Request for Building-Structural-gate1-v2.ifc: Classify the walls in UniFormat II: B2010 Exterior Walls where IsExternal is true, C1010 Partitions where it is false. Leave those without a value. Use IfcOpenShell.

First a look at what the model holds.

```python
import ifcopenshell
import ifcopenshell.util.element

model = ifcopenshell.open("Building-Structural-gate1-v2.ifc")
print(model.schema)
print("classifications:", [c.Name for c in model.by_type("IfcClassification")])
values = [ifcopenshell.util.element.get_pset(e, "Pset_WallCommon", "IsExternal") for e in model.by_type("IfcWall")]
for value in (True, False, None):
    print("IsExternal", value, values.count(value))
```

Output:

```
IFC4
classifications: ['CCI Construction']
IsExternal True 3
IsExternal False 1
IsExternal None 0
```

```python
import ifcopenshell
import ifcopenshell.api.classification
import ifcopenshell.util.element

model = ifcopenshell.open("Building-Structural-gate1-v2.ifc")

system = ifcopenshell.api.classification.add_classification(model, classification="UniFormat II")

walls = model.by_type("IfcWall")
external = {e: ifcopenshell.util.element.get_pset(e, "Pset_WallCommon", "IsExternal") for e in walls}
for flag, code, name in ((True, "B2010", "Exterior Walls"), (False, "C1010", "Partitions")):
    products = [e for e in walls if external[e] is flag]
    ifcopenshell.api.classification.add_reference(
        model, products=products, classification=system, identification=code, name=name
    )
    print(code, len(products))

model.write("Building-Structural-gate1-v2_edited.ifc")
```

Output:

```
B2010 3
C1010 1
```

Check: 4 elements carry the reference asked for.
